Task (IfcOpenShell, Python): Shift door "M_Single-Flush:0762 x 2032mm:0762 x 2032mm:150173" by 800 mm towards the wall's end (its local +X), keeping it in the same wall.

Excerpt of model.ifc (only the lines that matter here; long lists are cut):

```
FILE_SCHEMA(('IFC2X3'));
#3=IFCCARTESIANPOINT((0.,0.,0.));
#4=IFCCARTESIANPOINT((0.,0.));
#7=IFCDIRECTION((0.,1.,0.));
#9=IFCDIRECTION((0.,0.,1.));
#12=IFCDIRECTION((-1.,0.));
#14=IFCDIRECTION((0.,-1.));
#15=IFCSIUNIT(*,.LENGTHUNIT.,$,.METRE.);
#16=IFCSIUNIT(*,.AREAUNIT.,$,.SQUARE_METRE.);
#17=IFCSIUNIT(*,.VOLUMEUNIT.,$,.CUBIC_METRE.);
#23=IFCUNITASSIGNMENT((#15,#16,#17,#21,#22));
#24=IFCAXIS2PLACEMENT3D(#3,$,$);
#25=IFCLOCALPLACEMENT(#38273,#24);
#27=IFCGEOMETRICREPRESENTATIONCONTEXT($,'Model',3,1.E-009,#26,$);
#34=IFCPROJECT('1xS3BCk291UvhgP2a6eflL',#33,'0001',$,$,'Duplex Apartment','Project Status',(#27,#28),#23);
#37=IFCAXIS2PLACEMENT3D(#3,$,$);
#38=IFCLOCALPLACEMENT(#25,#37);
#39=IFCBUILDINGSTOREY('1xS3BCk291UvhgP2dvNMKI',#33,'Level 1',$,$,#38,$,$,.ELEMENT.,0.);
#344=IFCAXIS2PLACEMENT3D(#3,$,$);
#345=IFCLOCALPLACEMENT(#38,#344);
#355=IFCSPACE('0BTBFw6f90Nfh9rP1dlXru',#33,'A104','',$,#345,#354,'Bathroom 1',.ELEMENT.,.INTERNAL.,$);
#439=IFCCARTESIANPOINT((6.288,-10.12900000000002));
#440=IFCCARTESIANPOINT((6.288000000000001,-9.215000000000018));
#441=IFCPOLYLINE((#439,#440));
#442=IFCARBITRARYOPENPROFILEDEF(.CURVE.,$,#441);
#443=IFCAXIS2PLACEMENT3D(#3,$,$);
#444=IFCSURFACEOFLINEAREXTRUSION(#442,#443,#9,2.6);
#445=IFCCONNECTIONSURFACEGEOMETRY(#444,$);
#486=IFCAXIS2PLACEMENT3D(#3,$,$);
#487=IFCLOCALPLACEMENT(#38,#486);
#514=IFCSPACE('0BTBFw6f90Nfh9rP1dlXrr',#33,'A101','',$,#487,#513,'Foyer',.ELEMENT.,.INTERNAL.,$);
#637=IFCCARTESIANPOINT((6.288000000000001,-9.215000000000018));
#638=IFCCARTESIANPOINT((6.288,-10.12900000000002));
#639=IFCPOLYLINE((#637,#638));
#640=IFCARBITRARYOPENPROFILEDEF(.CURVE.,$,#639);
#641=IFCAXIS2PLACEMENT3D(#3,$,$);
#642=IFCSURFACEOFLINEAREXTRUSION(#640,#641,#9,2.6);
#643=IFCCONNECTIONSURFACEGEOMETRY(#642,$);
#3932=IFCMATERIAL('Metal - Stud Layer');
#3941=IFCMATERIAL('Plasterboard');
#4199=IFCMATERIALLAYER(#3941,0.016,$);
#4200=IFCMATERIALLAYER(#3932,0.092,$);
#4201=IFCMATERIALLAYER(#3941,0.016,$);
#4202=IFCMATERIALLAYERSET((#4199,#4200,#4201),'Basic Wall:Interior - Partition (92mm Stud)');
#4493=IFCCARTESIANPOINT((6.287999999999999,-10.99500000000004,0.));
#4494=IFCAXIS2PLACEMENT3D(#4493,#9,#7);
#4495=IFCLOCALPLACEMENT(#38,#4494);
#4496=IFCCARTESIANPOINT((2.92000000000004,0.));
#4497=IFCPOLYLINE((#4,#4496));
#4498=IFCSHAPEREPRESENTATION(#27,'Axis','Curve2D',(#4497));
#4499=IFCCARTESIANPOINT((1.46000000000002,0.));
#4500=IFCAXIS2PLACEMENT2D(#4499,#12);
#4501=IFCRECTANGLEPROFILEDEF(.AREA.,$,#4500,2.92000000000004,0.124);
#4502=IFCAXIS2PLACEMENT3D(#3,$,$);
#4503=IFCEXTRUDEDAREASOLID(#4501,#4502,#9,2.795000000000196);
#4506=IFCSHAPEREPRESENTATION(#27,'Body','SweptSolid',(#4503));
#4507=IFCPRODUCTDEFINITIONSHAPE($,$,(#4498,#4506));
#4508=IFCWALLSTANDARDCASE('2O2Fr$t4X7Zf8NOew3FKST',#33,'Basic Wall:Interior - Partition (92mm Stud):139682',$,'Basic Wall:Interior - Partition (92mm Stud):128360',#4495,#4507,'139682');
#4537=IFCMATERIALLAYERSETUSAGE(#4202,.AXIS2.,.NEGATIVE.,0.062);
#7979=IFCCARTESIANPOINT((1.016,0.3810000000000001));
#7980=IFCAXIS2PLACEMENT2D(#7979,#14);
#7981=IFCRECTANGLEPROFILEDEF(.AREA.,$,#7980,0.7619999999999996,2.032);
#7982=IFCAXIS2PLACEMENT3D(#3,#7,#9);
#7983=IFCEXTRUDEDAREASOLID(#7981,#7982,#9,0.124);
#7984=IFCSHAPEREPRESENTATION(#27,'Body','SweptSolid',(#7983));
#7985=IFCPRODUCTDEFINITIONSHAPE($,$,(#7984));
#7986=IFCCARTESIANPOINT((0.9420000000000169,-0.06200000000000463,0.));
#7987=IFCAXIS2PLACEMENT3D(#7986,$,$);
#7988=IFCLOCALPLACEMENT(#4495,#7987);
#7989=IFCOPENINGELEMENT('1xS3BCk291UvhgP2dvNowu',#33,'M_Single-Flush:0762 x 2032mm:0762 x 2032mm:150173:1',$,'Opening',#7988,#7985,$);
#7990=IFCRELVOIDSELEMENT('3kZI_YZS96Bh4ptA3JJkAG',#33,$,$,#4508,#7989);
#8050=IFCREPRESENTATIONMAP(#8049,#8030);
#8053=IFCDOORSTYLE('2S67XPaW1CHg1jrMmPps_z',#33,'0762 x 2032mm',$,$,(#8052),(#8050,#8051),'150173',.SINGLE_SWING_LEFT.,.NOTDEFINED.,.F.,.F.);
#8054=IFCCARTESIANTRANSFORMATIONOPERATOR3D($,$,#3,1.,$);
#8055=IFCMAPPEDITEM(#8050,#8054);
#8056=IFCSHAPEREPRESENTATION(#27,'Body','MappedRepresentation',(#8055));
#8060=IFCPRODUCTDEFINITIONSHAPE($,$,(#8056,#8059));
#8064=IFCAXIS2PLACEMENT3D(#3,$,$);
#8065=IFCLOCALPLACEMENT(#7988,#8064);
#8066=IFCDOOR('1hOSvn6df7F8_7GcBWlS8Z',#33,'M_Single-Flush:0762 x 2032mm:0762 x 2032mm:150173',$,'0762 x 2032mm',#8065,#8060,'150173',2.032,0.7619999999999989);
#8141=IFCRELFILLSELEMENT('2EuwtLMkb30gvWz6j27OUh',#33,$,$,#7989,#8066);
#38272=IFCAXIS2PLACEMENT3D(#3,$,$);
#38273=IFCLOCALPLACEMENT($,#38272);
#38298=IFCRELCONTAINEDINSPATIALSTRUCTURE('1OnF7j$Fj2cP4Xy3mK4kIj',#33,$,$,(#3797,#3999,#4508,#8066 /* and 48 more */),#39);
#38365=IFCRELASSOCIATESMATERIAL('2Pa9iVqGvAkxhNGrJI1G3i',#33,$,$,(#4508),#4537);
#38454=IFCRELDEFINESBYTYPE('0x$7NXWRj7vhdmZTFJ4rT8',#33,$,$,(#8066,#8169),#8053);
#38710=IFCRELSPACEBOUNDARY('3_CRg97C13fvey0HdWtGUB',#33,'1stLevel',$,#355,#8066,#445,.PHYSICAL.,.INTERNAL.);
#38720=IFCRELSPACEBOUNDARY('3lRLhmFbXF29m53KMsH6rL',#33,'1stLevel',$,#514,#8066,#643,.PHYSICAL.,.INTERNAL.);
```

```python
import numpy as np
import ifcopenshell
import ifcopenshell.api.geometry
import ifcopenshell.util.placement
import ifcopenshell.util.unit

model = ifcopenshell.open("model.ifc")
unit_scale = ifcopenshell.util.unit.calculate_unit_scale(model)

door = model.by_guid("1hOSvn6df7F8_7GcBWlS8Z")
opening = door.FillsVoids[0].RelatingOpeningElement
wall = opening.VoidsElements[0].RelatingBuildingElement

wall_matrix = ifcopenshell.util.placement.get_local_placement(wall.ObjectPlacement)
shift = wall_matrix[:3, 0] * 0.8 / unit_scale
before = ifcopenshell.util.placement.get_local_placement(door.ObjectPlacement)[:3, 3].copy()

# The door is placed relative to its opening, so it follows when the opening moves.
matrix = ifcopenshell.util.placement.get_local_placement(opening.ObjectPlacement)
matrix[:3, 3] += shift
ifcopenshell.api.geometry.edit_object_placement(
    model, product=opening, matrix=matrix, is_si=False, should_transform_children=True
)

# Space boundary surfaces are stored in each space's coordinates; move them too.
for rel in door.ProvidesBoundaries:
    if not rel.ConnectionGeometry:
        continue
    surface = rel.ConnectionGeometry.SurfaceOnRelatingElement
    space_matrix = ifcopenshell.util.placement.get_local_placement(rel.RelatingSpace.ObjectPlacement)
    point = np.array(surface.Position.Location.Coordinates) + space_matrix[:3, :3].T @ shift
    surface.Position = model.createIfcAxis2Placement3D(
        model.createIfcCartesianPoint(point.tolist()), surface.Position.Axis, surface.Position.RefDirection
    )

after = ifcopenshell.util.placement.get_local_placement(door.ObjectPlacement)[:3, 3]
print("door moved by", (after - before).round(3) + 0.0)

model.write("model_updated.ifc")
```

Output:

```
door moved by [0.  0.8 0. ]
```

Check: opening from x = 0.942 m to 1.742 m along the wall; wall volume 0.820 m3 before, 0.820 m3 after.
